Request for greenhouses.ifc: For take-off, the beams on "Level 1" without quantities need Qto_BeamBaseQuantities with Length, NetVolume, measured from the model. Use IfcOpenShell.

First a look at what the model holds.

```python
import ifcopenshell
import ifcopenshell.util.element
import ifcopenshell.util.unit

model = ifcopenshell.open("greenhouses.ifc")
print(model.schema)
for unit_type in ("LENGTHUNIT", "AREAUNIT", "VOLUMEUNIT"):
    print(unit_type, ifcopenshell.util.unit.calculate_unit_scale(model, unit_type))
storey = next(s for s in model.by_type("IfcBuildingStorey") if s.Name == "Level 1")
beams = [e for e in ifcopenshell.util.element.get_decomposition(storey) if e.is_a("IfcBeam")]
for e in sorted(beams, key=lambda e: e.id()):
    print(e.id(), e.is_a(), e.Name, list(ifcopenshell.util.element.get_psets(e, qtos_only=True)), sep=" | ")
```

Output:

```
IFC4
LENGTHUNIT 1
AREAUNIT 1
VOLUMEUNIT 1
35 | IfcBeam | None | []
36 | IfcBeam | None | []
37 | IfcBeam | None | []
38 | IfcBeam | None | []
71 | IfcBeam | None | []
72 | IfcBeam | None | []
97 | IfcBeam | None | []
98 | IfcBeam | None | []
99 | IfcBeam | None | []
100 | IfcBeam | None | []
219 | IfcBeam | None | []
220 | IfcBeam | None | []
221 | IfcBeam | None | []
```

```python
import ifcopenshell
import ifcopenshell.api.pset
import ifcopenshell.geom
import ifcopenshell.util.element
import ifcopenshell.util.shape
import ifcopenshell.util.unit

model = ifcopenshell.open("greenhouses.ifc")
unit_scale = ifcopenshell.util.unit.calculate_unit_scale(model)
volume_scale = ifcopenshell.util.unit.calculate_unit_scale(model, "VOLUMEUNIT")
settings = ifcopenshell.geom.settings()

storey = next(s for s in model.by_type("IfcBuildingStorey") if s.Name == "Level 1")
beams = [e for e in ifcopenshell.util.element.get_decomposition(storey) if e.is_a("IfcBeam")]

for e in sorted(beams, key=lambda e: e.id()):
    if ifcopenshell.util.element.get_psets(e, qtos_only=True, should_inherit=False):
        continue
    # Geometry comes back in metres, in the element's own axes.
    shape = ifcopenshell.geom.create_shape(settings, e)
    values = {
        "Length": ifcopenshell.util.shape.get_max_xyz(shape.geometry) / unit_scale,
        "NetVolume": ifcopenshell.util.shape.get_volume(shape.geometry) / volume_scale,
    }
    qto = ifcopenshell.api.pset.add_qto(model, product=e, name="Qto_BeamBaseQuantities")
    ifcopenshell.api.pset.edit_qto(model, qto=qto, properties=values)
    print(e.id(), {k: round(v, 3) for k, v in values.items()})

model.write("greenhouses-out.ifc")
```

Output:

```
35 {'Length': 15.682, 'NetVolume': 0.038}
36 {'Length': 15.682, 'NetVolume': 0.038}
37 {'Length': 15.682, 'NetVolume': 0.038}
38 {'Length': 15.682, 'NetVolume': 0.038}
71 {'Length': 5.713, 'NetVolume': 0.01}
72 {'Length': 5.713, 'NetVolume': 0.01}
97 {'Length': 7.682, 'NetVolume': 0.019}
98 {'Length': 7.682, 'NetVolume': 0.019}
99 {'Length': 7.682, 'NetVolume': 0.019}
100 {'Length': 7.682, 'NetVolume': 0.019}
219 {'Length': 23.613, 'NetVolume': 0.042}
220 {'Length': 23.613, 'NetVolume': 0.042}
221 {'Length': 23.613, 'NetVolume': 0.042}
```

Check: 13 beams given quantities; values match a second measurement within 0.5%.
